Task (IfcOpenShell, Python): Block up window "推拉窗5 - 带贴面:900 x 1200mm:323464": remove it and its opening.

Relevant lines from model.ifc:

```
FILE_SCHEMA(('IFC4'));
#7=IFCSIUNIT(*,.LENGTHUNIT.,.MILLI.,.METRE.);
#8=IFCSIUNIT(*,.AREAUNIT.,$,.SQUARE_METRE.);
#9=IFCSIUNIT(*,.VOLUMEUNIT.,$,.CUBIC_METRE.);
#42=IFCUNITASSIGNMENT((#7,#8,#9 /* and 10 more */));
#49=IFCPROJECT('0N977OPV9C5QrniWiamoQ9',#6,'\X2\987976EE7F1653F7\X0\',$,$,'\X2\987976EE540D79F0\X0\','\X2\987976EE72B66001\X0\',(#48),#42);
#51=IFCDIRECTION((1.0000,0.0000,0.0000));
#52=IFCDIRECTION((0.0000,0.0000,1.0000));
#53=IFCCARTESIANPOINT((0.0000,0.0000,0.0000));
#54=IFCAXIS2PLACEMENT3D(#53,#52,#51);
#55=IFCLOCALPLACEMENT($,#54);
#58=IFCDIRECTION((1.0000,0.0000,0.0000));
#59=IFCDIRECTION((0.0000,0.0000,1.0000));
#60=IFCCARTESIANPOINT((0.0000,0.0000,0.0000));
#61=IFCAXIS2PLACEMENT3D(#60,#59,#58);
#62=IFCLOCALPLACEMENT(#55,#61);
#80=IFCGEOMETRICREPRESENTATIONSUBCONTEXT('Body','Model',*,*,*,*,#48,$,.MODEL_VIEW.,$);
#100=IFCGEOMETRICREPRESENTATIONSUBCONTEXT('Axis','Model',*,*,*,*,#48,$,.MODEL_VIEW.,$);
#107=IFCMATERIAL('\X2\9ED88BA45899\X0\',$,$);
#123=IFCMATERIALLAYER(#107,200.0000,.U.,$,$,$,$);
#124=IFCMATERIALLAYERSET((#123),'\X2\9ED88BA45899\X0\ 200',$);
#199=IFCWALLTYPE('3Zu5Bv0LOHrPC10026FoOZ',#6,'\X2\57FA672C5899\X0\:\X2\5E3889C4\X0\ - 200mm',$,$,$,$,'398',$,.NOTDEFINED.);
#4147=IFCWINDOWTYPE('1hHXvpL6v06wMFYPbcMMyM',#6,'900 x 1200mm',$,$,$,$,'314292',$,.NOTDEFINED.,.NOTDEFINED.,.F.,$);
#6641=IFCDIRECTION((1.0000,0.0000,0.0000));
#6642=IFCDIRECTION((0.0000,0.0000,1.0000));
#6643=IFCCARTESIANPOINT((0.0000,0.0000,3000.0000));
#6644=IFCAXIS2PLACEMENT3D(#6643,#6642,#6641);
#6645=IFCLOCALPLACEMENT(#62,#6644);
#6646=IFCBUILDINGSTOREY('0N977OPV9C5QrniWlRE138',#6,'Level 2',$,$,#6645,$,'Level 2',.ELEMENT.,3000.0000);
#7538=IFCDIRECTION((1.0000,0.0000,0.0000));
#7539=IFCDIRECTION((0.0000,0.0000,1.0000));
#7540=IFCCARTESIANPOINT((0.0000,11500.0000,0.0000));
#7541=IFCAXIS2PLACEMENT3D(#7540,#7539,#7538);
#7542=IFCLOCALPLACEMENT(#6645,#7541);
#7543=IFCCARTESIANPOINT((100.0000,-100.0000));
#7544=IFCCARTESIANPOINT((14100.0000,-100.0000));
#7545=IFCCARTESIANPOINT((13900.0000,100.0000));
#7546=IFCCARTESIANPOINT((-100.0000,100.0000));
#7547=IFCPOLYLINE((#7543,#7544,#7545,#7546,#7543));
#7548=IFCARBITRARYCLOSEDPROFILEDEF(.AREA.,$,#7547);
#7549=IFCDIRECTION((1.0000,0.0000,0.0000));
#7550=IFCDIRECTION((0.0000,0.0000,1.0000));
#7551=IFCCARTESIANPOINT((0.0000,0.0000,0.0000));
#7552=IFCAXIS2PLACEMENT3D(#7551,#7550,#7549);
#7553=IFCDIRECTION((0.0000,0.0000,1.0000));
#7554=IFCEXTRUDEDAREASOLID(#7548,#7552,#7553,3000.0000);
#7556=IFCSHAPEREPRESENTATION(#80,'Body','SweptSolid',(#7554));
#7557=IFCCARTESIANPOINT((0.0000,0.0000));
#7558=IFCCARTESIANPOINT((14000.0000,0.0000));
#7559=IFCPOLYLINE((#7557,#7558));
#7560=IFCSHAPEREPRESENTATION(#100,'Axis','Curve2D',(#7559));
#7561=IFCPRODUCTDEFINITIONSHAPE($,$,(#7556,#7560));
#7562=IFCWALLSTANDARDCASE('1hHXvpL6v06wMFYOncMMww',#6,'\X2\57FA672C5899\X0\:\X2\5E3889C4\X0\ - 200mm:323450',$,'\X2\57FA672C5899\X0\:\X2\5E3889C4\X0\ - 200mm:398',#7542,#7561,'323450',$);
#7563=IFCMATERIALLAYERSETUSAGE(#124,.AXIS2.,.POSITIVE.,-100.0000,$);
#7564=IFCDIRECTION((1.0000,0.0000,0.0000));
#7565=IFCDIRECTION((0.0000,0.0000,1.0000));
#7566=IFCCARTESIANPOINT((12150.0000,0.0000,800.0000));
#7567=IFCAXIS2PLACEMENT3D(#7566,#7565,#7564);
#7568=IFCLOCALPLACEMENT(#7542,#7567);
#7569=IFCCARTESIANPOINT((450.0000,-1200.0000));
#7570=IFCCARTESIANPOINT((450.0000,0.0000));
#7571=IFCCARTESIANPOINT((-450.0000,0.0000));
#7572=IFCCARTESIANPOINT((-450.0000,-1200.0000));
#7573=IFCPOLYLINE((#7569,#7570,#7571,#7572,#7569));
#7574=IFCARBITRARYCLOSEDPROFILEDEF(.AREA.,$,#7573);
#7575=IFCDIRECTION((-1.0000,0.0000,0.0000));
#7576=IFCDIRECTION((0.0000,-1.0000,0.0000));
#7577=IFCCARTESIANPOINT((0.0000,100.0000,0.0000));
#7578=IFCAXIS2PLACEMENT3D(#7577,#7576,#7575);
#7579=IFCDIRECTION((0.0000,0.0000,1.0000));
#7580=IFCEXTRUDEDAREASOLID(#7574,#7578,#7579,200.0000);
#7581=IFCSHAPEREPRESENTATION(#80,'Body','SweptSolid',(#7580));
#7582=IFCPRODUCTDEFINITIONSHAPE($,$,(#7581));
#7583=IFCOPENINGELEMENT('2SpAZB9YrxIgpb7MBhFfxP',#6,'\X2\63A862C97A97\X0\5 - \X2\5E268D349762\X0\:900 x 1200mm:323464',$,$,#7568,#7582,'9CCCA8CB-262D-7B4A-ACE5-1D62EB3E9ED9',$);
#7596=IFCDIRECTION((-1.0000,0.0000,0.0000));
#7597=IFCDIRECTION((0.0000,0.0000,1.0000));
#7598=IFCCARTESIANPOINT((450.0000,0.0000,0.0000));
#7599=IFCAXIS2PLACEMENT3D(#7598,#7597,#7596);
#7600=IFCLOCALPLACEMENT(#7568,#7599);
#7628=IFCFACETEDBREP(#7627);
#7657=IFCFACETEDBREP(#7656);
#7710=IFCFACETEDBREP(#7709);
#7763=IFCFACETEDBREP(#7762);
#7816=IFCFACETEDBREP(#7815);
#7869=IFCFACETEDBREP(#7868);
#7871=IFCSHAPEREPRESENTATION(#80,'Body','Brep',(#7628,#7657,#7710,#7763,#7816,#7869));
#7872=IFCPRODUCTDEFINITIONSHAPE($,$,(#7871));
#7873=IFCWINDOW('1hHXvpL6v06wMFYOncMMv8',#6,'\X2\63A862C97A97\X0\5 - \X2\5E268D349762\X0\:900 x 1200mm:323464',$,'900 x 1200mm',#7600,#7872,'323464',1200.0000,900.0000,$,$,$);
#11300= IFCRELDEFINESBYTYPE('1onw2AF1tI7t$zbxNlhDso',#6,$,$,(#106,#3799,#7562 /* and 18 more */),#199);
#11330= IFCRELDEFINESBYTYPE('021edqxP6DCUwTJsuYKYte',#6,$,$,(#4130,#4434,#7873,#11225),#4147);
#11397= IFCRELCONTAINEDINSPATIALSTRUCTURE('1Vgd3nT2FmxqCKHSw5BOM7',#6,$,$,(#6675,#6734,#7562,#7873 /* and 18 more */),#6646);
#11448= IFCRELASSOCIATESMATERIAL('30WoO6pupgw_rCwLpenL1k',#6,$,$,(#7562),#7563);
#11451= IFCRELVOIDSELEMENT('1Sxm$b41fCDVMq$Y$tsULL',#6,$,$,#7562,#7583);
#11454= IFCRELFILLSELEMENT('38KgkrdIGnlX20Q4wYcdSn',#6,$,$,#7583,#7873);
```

```python
import ifcopenshell
import ifcopenshell.api.feature
import ifcopenshell.api.root
import ifcopenshell.geom
import ifcopenshell.util.shape

model = ifcopenshell.open("model.ifc")
settings = ifcopenshell.geom.settings()


def volume(element):
    """Net volume in cubic metres, openings subtracted."""
    shape = ifcopenshell.geom.create_shape(settings, element)
    return ifcopenshell.util.shape.get_volume(shape.geometry)


window = model.by_id(7873)
opening = window.FillsVoids[0].RelatingOpeningElement
wall = opening.VoidsElements[0].RelatingBuildingElement
before = volume(wall)

ifcopenshell.api.root.remove_product(model, product=window)
ifcopenshell.api.feature.remove_feature(model, feature=opening)

after = volume(wall)

print(f"wall volume {before:.3f} -> {after:.3f} m3")

model.write("model_rev.ifc")
```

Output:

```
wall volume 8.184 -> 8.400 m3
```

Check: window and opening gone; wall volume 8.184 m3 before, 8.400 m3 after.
